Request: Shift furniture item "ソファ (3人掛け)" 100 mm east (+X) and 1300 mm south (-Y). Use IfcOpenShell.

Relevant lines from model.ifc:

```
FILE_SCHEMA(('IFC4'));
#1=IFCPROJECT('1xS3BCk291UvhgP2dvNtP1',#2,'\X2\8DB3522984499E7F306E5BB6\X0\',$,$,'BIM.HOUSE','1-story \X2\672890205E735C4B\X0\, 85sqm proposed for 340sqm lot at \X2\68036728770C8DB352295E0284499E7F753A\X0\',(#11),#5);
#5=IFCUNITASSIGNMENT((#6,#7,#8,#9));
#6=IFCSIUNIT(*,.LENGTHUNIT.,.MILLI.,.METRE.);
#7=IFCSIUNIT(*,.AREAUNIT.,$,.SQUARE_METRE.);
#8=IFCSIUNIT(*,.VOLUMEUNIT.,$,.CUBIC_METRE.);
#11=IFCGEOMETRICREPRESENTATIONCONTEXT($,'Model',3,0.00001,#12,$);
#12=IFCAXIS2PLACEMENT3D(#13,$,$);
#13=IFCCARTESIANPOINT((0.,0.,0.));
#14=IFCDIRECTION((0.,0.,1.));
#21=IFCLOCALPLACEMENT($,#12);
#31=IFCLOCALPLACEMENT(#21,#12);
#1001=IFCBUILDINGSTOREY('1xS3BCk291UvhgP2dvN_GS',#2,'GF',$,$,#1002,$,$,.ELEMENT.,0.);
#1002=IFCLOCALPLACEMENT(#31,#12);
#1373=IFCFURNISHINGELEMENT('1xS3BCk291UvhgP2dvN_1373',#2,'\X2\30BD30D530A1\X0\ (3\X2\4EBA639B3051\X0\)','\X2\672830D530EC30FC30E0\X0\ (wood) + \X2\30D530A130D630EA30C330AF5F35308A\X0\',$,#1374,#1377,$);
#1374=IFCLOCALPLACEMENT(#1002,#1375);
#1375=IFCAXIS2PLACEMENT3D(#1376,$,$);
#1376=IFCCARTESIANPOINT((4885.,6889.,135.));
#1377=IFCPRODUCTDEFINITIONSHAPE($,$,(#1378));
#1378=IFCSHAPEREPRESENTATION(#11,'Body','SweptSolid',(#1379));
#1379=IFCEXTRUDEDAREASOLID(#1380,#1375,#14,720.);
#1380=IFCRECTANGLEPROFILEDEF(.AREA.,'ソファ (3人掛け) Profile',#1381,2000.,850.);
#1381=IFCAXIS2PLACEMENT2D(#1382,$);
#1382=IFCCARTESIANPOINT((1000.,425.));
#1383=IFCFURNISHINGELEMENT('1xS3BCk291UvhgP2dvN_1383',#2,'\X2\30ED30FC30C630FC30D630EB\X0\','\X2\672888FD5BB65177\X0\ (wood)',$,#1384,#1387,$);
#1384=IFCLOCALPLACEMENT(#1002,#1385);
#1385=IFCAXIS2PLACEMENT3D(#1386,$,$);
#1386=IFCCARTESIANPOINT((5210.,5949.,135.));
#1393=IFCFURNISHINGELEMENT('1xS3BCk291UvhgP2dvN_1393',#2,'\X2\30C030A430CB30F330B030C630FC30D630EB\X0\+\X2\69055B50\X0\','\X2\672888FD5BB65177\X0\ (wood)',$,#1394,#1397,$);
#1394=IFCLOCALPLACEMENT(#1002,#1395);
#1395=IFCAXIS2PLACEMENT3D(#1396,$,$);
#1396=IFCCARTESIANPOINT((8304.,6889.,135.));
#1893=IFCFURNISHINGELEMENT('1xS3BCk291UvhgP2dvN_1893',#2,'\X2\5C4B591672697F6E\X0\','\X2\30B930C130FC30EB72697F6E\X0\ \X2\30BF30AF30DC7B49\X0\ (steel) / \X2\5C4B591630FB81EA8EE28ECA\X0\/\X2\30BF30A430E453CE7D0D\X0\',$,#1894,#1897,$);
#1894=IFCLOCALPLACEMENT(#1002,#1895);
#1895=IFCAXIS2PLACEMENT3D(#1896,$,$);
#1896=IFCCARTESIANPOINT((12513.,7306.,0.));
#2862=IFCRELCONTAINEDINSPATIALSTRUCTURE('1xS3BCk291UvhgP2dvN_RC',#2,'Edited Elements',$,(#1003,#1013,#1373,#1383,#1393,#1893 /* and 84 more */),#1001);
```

```python
import ifcopenshell
import ifcopenshell.api.geometry
import ifcopenshell.util.placement

model = ifcopenshell.open("model.ifc")

item = model.by_guid("1xS3BCk291UvhgP2dvN_1373")
matrix = ifcopenshell.util.placement.get_local_placement(item.ObjectPlacement)
matrix[0, 3] += 100.0
matrix[1, 3] -= 1300.0
ifcopenshell.api.geometry.edit_object_placement(model, product=item, matrix=matrix, is_si=False)

print(ifcopenshell.util.placement.get_local_placement(item.ObjectPlacement).round(3) + 0.0)

model.write("model_updated.ifc")
```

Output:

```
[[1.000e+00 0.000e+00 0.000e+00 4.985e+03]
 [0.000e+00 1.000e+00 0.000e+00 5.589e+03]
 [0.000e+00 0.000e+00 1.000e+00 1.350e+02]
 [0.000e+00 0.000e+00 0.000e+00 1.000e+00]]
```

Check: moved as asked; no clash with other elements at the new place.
